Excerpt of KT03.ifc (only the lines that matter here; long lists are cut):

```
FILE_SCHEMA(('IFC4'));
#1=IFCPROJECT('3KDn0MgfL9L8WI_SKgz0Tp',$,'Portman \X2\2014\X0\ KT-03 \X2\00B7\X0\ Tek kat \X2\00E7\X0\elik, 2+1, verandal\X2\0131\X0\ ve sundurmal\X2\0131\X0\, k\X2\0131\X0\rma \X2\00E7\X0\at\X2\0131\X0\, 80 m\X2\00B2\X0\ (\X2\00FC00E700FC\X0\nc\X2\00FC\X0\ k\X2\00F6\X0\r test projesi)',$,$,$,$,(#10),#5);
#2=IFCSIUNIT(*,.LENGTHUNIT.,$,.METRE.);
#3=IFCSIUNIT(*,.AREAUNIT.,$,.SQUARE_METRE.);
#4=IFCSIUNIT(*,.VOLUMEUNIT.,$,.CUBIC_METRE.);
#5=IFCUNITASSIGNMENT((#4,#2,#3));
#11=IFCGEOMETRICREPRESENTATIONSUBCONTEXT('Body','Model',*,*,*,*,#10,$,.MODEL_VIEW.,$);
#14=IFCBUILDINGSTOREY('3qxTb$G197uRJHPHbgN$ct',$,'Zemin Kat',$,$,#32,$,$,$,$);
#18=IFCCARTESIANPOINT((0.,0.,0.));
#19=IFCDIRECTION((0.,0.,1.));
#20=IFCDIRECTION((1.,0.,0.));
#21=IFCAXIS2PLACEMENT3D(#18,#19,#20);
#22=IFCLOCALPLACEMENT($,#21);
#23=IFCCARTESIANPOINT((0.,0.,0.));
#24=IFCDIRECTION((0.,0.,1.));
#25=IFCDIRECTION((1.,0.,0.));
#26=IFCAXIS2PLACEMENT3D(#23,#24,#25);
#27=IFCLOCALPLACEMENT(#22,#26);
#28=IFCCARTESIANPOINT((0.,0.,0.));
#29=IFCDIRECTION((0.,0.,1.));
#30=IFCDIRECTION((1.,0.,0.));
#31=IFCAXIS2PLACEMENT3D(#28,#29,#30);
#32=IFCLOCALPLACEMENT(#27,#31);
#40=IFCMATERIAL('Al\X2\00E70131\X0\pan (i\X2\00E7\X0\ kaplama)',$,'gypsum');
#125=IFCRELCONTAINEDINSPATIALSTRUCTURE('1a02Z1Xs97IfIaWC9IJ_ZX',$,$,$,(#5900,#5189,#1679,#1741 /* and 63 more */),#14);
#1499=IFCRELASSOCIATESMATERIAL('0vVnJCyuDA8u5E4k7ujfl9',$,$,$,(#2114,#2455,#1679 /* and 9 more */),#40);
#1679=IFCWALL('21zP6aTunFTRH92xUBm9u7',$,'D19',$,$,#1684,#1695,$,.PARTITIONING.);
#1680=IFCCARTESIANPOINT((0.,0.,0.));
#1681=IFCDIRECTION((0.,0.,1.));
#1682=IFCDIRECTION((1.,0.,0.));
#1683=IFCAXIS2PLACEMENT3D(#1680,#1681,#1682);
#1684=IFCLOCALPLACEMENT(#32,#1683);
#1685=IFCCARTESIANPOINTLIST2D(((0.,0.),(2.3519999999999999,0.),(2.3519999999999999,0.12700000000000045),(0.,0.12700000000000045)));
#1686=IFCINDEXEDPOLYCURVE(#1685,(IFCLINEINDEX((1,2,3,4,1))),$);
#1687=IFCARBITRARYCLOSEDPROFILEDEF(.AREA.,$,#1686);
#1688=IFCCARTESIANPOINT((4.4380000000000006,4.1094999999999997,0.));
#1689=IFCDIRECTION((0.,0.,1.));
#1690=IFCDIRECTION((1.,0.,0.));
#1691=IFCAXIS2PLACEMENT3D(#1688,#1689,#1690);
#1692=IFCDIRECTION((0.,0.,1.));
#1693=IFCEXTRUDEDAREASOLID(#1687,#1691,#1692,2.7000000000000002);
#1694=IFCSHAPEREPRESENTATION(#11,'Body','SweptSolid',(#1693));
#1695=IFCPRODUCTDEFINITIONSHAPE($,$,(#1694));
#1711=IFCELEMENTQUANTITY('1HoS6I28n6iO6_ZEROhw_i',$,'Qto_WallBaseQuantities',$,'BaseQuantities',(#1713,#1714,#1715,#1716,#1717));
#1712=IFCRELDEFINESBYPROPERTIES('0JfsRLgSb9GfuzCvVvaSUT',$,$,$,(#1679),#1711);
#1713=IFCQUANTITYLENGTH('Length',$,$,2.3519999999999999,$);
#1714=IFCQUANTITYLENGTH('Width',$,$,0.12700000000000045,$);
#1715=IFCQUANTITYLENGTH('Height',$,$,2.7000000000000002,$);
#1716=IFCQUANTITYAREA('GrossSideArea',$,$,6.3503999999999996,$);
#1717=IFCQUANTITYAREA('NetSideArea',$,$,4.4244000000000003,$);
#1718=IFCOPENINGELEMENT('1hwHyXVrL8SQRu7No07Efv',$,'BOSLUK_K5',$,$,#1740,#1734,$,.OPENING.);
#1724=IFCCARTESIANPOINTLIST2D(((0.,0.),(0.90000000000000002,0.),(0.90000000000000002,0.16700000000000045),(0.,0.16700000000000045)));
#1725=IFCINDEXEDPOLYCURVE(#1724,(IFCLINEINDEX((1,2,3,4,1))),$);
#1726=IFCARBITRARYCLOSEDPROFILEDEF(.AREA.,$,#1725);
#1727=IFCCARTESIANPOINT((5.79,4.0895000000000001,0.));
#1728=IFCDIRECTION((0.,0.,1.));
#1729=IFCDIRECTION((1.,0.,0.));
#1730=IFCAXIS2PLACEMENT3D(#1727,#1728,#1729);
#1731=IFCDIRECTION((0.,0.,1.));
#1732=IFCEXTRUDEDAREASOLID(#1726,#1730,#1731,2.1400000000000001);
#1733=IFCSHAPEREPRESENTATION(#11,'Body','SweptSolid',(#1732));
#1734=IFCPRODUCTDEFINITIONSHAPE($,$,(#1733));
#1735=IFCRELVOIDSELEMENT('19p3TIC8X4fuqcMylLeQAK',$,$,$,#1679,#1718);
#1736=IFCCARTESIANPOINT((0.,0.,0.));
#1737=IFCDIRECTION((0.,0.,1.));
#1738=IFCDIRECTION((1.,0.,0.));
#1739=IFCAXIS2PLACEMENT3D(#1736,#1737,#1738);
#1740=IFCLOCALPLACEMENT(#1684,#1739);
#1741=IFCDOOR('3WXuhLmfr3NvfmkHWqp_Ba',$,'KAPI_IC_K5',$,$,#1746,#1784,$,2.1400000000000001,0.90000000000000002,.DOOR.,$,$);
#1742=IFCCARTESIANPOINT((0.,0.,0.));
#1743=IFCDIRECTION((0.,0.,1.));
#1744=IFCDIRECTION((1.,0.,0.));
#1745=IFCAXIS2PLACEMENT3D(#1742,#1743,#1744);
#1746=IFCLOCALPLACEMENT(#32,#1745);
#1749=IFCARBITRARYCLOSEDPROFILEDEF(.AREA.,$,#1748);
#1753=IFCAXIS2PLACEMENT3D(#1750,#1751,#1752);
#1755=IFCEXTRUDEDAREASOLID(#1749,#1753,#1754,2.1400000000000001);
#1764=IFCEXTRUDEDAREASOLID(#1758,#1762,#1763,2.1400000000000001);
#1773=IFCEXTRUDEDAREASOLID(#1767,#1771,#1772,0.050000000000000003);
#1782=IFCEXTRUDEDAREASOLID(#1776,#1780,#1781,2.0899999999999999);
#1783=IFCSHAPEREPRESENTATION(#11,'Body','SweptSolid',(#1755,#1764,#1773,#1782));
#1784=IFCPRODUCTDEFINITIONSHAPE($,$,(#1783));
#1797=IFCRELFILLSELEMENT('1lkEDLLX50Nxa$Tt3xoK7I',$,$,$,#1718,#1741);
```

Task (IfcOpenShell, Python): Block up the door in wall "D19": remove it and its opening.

```python
import ifcopenshell
import ifcopenshell.api.feature
import ifcopenshell.api.pset
import ifcopenshell.api.root
import ifcopenshell.geom
import ifcopenshell.util.element
import ifcopenshell.util.shape
import ifcopenshell.util.unit

model = ifcopenshell.open("KT03.ifc")
area_scale = ifcopenshell.util.unit.calculate_unit_scale(model, "AREAUNIT")
settings = ifcopenshell.geom.settings()


def volume(element):
    """Net volume in cubic metres, openings subtracted."""
    shape = ifcopenshell.geom.create_shape(settings, element)
    return ifcopenshell.util.shape.get_volume(shape.geometry)


door = model.by_id(1741)
opening = door.FillsVoids[0].RelatingOpeningElement
wall = opening.VoidsElements[0].RelatingBuildingElement
before = volume(wall)

ifcopenshell.api.root.remove_product(model, product=door)
ifcopenshell.api.feature.remove_feature(model, feature=opening)

after = volume(wall)
thickness = 0.127  # wall thickness in metres

# Update the wall's stored quantities.
qto = model.by_id(ifcopenshell.util.element.get_pset(wall, "Qto_WallBaseQuantities", should_inherit=False)["id"])
ifcopenshell.api.pset.edit_qto(model, qto=qto, properties={"NetSideArea": after / thickness / area_scale})

print(f"wall volume {before:.3f} -> {after:.3f} m3")

model.write("KT03_updated.ifc")
```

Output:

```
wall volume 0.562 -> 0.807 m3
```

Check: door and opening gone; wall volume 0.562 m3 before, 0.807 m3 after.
